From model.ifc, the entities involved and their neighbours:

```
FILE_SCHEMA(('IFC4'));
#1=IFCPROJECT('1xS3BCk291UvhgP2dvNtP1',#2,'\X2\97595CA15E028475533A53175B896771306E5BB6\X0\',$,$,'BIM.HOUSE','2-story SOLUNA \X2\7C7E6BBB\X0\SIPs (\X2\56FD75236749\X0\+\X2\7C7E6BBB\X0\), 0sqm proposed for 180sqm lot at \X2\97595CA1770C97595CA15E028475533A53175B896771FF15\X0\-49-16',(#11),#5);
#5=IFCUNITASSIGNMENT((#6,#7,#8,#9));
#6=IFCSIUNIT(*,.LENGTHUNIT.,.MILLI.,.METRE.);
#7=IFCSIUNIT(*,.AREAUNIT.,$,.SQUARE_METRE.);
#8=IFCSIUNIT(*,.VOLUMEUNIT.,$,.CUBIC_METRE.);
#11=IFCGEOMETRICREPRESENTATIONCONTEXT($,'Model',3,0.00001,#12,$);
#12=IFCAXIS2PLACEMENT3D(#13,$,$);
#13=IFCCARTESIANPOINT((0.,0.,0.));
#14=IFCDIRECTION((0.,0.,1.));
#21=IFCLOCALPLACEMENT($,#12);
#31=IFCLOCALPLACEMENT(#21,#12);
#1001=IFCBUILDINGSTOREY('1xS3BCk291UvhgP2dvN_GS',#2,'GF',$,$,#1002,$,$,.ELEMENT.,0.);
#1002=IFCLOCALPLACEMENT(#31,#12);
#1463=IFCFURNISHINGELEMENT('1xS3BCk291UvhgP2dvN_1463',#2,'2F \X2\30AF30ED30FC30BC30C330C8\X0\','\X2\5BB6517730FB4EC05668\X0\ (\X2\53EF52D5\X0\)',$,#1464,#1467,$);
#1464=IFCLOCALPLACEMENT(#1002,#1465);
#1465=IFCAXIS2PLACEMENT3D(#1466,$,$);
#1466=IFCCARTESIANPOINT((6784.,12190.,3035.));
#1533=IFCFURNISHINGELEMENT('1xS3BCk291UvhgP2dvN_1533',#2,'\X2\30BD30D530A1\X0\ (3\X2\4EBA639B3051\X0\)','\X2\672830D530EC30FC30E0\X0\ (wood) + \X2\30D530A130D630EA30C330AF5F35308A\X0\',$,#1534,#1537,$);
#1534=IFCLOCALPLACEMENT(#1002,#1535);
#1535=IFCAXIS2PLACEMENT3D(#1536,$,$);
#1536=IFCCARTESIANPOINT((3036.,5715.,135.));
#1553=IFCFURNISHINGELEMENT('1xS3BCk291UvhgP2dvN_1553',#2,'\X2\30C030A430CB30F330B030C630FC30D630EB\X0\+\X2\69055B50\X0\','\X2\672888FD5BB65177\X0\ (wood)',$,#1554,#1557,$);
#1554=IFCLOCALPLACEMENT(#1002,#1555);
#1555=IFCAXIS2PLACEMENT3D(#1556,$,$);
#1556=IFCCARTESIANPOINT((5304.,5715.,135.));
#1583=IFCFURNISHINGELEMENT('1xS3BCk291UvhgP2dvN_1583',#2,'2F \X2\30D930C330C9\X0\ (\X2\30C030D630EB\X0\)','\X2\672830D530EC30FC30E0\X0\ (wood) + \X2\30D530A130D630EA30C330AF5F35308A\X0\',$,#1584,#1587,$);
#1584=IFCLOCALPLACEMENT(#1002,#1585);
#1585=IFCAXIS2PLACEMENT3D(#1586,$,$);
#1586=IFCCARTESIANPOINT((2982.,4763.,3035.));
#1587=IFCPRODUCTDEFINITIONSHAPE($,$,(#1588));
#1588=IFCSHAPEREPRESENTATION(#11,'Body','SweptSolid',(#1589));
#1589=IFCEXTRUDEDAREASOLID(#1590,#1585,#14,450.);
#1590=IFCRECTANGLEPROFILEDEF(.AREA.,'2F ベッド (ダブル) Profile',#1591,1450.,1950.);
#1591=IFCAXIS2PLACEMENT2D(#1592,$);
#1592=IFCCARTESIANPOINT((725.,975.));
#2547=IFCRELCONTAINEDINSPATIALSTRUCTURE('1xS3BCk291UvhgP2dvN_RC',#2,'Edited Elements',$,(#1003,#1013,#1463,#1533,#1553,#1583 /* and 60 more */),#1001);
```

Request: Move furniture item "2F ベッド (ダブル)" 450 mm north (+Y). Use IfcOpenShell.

```python
import ifcopenshell
import ifcopenshell.api.geometry
import ifcopenshell.util.placement

model = ifcopenshell.open("model.ifc")

item = model.by_guid("1xS3BCk291UvhgP2dvN_1583")
matrix = ifcopenshell.util.placement.get_local_placement(item.ObjectPlacement)
matrix[1, 3] += 450.0
ifcopenshell.api.geometry.edit_object_placement(model, product=item, matrix=matrix, is_si=False)

print(ifcopenshell.util.placement.get_local_placement(item.ObjectPlacement).round(3) + 0.0)

model.write("model_v2.ifc")
```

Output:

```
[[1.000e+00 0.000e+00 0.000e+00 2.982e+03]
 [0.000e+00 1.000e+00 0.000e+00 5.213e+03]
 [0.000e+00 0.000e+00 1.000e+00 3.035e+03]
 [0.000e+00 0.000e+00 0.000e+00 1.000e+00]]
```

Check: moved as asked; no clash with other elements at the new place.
